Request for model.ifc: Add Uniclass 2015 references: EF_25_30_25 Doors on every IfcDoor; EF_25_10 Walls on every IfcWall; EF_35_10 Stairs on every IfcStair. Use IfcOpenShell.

First a look at what the model holds.

```python
import ifcopenshell

model = ifcopenshell.open("model.ifc")
print(model.schema)
print("classifications:", [c.Name for c in model.by_type("IfcClassification")])
for ifc_class in ("IfcDoor", "IfcRoof", "IfcStair", "IfcWall", "IfcWindow"):
    print(ifc_class, len(model.by_type(ifc_class)))
```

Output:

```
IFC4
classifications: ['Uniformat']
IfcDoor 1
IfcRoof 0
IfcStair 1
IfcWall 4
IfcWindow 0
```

```python
import ifcopenshell
import ifcopenshell.api.classification

model = ifcopenshell.open("model.ifc")

system = ifcopenshell.api.classification.add_classification(model, classification="Uniclass 2015")

codes = {
    "IfcDoor": ("EF_25_30_25", "Doors"),
    "IfcWall": ("EF_25_10", "Walls"),
    "IfcStair": ("EF_35_10", "Stairs"),
}
for ifc_class, (code, name) in codes.items():
    products = model.by_type(ifc_class)
    ifcopenshell.api.classification.add_reference(
        model, products=products, classification=system, identification=code, name=name
    )
    print(code, len(products))

model.write("model_updated.ifc")
```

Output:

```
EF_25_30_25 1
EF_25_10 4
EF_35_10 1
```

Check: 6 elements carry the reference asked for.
